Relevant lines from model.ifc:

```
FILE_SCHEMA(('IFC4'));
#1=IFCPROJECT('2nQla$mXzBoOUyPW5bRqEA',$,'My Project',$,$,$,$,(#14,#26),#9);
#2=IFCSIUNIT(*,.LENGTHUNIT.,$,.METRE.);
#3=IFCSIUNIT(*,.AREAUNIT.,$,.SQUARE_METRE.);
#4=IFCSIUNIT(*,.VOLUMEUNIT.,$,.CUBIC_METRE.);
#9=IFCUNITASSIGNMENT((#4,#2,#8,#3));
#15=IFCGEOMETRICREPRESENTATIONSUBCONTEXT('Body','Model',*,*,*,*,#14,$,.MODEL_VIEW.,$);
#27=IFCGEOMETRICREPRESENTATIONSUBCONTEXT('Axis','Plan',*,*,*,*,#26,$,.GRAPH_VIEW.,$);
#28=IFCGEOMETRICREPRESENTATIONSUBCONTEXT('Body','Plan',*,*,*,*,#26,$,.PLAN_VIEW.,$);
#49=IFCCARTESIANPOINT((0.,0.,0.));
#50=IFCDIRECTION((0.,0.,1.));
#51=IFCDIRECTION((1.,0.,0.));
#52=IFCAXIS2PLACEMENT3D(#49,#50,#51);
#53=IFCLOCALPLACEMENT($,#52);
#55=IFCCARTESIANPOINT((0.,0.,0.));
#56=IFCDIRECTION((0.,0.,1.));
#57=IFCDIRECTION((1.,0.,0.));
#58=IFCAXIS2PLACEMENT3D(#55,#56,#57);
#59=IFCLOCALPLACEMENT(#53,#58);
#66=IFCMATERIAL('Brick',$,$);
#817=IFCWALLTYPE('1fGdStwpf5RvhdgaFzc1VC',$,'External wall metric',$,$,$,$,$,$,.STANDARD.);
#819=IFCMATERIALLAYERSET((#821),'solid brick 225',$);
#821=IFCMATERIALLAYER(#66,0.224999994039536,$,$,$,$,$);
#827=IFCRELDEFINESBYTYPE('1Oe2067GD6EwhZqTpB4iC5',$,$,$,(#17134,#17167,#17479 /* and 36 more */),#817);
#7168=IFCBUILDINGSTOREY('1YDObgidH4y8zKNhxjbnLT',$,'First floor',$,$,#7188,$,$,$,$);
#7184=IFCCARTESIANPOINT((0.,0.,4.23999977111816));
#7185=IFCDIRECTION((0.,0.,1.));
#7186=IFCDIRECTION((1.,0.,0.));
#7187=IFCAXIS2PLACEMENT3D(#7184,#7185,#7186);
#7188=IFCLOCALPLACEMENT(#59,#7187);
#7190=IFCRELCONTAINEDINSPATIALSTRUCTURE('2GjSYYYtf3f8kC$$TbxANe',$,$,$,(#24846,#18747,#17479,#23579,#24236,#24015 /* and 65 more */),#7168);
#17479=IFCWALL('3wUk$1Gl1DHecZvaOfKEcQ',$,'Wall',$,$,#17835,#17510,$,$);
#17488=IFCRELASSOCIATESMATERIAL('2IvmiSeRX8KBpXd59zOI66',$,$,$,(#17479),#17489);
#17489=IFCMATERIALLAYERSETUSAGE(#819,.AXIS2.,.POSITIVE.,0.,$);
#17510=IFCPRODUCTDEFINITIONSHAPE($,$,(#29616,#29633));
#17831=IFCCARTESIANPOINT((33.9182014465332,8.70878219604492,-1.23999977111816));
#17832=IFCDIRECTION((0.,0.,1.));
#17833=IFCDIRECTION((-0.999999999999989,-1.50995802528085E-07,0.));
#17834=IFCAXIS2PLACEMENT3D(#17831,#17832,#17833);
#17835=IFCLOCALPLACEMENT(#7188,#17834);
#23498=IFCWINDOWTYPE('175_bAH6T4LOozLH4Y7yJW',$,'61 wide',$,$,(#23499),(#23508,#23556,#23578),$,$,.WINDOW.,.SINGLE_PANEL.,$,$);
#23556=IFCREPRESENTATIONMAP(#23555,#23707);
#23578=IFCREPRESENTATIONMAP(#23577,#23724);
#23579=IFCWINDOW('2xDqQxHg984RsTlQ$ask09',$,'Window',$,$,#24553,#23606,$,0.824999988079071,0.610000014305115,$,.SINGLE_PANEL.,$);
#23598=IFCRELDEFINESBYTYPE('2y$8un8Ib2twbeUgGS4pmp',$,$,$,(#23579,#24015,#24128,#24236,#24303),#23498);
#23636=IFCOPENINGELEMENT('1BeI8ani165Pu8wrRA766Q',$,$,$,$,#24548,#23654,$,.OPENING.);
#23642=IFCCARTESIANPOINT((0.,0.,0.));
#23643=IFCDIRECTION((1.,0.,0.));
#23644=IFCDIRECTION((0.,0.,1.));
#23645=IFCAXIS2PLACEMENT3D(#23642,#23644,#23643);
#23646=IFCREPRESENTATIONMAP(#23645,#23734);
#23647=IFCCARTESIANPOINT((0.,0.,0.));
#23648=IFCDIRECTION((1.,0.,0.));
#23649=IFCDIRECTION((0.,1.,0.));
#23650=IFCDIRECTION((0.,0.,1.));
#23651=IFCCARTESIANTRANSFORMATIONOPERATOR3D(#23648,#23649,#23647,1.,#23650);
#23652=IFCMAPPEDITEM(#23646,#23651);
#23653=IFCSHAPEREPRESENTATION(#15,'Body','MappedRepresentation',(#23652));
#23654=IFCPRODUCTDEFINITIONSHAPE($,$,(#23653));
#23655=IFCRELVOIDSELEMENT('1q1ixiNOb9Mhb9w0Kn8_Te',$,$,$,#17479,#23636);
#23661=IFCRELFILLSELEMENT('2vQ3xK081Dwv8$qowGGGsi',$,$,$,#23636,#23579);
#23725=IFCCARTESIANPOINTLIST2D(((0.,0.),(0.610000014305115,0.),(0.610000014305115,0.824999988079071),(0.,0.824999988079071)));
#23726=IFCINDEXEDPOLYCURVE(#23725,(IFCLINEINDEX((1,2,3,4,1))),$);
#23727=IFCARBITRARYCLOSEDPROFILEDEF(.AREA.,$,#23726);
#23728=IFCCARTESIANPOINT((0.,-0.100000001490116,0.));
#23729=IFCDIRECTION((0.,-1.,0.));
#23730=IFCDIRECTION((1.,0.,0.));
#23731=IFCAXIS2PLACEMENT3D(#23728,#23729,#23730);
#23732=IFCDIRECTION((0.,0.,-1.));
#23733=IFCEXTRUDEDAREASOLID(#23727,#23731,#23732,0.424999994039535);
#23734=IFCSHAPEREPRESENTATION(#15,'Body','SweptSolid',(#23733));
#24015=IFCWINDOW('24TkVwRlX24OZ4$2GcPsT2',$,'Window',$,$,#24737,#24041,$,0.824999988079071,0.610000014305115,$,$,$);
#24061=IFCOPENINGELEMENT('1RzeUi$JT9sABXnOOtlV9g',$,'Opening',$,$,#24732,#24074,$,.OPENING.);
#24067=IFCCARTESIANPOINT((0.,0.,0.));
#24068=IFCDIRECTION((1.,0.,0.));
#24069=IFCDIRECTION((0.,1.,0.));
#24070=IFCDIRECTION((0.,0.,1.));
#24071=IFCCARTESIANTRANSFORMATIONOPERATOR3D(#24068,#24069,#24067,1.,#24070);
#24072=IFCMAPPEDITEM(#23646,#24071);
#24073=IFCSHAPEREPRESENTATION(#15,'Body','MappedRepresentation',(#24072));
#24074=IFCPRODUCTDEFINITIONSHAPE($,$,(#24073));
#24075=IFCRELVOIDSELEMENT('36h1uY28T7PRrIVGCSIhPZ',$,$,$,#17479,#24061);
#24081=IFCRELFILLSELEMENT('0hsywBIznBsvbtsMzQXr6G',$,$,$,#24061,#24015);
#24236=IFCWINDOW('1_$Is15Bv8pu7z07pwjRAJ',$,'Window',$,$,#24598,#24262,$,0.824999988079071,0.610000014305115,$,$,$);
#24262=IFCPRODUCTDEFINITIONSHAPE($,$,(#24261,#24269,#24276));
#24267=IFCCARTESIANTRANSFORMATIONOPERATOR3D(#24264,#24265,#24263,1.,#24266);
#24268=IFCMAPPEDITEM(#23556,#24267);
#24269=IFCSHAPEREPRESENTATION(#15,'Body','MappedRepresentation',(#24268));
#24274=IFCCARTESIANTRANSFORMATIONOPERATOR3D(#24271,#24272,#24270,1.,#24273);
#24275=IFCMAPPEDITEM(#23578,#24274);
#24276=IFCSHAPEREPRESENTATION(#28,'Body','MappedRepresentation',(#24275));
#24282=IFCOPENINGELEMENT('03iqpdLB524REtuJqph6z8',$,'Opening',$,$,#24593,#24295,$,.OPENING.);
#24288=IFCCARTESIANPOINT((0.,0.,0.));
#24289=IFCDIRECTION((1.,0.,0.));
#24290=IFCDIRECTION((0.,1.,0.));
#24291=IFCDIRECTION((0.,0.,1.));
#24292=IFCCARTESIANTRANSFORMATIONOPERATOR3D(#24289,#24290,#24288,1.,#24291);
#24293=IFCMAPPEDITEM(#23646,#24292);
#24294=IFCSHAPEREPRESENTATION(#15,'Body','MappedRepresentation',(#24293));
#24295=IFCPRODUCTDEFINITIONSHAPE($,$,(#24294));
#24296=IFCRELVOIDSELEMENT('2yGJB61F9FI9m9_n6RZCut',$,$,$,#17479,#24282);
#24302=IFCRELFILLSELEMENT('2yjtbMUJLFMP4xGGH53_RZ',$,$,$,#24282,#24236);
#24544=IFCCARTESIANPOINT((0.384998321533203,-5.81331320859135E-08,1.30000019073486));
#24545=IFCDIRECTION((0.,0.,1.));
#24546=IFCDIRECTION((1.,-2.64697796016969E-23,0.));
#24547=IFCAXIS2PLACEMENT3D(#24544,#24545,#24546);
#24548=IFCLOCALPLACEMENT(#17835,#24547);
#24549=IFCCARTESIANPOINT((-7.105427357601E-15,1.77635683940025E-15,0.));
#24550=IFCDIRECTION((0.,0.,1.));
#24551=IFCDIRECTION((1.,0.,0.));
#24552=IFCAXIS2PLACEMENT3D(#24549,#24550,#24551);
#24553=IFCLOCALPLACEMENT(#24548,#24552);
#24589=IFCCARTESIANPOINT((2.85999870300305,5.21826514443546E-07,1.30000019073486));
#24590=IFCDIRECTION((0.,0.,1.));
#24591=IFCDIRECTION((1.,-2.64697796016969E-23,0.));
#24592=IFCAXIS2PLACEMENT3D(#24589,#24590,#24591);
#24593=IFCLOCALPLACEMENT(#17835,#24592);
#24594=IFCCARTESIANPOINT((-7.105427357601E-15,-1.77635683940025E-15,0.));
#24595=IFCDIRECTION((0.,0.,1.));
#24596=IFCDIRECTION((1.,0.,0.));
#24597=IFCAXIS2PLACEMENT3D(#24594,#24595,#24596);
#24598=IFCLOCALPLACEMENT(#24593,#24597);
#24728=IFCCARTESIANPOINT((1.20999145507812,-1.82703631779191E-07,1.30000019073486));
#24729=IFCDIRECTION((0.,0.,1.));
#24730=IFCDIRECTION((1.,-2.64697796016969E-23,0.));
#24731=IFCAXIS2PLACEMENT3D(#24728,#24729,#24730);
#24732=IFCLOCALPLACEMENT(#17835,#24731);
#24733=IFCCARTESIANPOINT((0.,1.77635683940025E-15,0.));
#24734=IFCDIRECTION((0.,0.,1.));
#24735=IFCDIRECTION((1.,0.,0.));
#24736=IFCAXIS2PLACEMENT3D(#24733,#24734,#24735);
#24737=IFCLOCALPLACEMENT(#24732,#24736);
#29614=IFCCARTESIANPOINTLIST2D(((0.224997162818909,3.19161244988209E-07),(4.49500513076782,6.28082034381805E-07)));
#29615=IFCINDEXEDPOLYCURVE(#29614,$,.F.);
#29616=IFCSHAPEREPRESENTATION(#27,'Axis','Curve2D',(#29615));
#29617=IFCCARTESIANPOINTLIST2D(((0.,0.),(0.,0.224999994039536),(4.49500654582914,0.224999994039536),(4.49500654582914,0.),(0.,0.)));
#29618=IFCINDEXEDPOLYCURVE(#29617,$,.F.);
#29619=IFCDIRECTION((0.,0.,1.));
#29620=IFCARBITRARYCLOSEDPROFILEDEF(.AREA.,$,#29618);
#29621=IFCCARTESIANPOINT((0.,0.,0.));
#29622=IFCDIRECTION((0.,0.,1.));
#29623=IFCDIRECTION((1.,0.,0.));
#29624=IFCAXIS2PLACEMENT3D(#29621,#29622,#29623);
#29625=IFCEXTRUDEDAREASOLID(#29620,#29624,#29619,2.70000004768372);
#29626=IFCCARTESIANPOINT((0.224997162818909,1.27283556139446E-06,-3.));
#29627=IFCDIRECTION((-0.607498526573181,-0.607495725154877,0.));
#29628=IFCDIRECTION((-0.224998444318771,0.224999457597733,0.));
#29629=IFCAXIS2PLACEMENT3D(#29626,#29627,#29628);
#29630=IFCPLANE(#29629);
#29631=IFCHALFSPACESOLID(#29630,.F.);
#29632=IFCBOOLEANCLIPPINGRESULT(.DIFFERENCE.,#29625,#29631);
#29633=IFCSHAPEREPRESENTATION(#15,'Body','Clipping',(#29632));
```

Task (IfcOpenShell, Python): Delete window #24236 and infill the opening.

```python
import ifcopenshell
import ifcopenshell.api.feature
import ifcopenshell.api.root
import ifcopenshell.geom
import ifcopenshell.util.shape

model = ifcopenshell.open("model.ifc")
settings = ifcopenshell.geom.settings()


def volume(element):
    """Net volume in cubic metres, openings subtracted."""
    shape = ifcopenshell.geom.create_shape(settings, element)
    return ifcopenshell.util.shape.get_volume(shape.geometry)


window = model.by_guid("1_$Is15Bv8pu7z07pwjRAJ")
opening = window.FillsVoids[0].RelatingOpeningElement
wall = opening.VoidsElements[0].RelatingBuildingElement
before = volume(wall)

ifcopenshell.api.root.remove_product(model, product=window)
ifcopenshell.api.feature.remove_feature(model, feature=opening)

after = volume(wall)

print(f"wall volume {before:.3f} -> {after:.3f} m3")

model.write("model_updated.ifc")
```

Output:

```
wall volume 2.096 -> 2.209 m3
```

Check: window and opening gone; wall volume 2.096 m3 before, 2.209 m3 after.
